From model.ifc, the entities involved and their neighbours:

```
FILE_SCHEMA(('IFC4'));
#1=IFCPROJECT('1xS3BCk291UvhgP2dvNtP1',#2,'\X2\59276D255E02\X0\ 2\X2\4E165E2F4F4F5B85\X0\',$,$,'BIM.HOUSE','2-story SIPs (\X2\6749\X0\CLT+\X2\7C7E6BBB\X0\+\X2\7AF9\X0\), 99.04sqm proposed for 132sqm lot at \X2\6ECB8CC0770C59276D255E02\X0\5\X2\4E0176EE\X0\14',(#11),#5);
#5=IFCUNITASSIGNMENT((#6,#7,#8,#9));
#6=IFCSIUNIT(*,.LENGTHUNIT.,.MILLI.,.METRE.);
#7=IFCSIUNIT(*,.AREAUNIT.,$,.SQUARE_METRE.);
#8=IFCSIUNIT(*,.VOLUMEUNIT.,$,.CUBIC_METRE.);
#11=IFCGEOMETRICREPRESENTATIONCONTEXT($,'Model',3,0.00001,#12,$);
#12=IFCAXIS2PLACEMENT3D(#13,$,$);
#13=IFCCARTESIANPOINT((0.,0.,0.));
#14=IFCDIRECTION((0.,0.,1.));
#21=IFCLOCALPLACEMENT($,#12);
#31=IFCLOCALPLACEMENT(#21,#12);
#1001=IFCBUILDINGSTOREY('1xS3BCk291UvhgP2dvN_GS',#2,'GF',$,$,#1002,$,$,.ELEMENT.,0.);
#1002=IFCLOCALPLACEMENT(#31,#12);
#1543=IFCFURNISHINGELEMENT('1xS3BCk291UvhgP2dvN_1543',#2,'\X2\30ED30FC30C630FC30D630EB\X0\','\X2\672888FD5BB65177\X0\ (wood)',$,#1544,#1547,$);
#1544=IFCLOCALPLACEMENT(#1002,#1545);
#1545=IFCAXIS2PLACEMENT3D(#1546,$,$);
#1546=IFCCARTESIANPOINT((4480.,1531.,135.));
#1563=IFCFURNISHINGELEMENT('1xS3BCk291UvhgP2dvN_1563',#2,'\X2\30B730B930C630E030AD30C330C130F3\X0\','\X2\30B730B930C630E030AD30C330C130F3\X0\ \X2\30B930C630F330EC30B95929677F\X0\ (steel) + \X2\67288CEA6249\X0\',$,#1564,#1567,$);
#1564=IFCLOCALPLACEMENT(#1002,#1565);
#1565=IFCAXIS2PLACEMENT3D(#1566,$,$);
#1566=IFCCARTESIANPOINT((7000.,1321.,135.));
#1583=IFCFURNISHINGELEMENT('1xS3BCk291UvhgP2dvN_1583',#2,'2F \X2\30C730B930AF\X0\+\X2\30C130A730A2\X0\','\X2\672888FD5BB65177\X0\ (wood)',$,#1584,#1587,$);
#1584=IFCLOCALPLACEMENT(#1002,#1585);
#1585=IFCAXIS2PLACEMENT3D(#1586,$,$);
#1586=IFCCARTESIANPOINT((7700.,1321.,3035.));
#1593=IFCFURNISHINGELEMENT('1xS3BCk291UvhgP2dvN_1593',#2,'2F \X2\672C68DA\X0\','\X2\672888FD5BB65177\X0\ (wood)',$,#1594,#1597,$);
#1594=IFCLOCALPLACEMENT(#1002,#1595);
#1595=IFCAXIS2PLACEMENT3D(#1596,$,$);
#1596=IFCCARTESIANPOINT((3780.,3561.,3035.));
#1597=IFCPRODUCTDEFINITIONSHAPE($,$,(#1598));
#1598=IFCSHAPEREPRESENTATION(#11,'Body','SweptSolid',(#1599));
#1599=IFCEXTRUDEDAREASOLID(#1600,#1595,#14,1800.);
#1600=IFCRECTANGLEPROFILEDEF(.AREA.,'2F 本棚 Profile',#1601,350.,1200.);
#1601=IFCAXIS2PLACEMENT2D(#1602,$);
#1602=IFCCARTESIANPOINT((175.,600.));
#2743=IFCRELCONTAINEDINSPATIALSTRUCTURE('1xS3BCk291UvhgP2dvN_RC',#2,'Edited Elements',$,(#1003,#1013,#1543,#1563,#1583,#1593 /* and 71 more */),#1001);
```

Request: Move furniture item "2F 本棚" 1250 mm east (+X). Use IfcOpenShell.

```python
import ifcopenshell
import ifcopenshell.api.geometry
import ifcopenshell.util.placement
import ifcopenshell.util.unit

model = ifcopenshell.open("model.ifc")
unit_scale = ifcopenshell.util.unit.calculate_unit_scale(model)

item = model.by_guid("1xS3BCk291UvhgP2dvN_1593")
matrix = ifcopenshell.util.placement.get_local_placement(item.ObjectPlacement)
matrix[0, 3] += 1.25 / unit_scale
ifcopenshell.api.geometry.edit_object_placement(model, product=item, matrix=matrix, is_si=False)

print(ifcopenshell.util.placement.get_local_placement(item.ObjectPlacement).round(3) + 0.0)

model.write("model_updated.ifc")
```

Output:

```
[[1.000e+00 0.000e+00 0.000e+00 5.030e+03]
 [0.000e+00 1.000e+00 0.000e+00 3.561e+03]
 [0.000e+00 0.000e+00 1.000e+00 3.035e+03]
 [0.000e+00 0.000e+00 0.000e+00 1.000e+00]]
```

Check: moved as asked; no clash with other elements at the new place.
